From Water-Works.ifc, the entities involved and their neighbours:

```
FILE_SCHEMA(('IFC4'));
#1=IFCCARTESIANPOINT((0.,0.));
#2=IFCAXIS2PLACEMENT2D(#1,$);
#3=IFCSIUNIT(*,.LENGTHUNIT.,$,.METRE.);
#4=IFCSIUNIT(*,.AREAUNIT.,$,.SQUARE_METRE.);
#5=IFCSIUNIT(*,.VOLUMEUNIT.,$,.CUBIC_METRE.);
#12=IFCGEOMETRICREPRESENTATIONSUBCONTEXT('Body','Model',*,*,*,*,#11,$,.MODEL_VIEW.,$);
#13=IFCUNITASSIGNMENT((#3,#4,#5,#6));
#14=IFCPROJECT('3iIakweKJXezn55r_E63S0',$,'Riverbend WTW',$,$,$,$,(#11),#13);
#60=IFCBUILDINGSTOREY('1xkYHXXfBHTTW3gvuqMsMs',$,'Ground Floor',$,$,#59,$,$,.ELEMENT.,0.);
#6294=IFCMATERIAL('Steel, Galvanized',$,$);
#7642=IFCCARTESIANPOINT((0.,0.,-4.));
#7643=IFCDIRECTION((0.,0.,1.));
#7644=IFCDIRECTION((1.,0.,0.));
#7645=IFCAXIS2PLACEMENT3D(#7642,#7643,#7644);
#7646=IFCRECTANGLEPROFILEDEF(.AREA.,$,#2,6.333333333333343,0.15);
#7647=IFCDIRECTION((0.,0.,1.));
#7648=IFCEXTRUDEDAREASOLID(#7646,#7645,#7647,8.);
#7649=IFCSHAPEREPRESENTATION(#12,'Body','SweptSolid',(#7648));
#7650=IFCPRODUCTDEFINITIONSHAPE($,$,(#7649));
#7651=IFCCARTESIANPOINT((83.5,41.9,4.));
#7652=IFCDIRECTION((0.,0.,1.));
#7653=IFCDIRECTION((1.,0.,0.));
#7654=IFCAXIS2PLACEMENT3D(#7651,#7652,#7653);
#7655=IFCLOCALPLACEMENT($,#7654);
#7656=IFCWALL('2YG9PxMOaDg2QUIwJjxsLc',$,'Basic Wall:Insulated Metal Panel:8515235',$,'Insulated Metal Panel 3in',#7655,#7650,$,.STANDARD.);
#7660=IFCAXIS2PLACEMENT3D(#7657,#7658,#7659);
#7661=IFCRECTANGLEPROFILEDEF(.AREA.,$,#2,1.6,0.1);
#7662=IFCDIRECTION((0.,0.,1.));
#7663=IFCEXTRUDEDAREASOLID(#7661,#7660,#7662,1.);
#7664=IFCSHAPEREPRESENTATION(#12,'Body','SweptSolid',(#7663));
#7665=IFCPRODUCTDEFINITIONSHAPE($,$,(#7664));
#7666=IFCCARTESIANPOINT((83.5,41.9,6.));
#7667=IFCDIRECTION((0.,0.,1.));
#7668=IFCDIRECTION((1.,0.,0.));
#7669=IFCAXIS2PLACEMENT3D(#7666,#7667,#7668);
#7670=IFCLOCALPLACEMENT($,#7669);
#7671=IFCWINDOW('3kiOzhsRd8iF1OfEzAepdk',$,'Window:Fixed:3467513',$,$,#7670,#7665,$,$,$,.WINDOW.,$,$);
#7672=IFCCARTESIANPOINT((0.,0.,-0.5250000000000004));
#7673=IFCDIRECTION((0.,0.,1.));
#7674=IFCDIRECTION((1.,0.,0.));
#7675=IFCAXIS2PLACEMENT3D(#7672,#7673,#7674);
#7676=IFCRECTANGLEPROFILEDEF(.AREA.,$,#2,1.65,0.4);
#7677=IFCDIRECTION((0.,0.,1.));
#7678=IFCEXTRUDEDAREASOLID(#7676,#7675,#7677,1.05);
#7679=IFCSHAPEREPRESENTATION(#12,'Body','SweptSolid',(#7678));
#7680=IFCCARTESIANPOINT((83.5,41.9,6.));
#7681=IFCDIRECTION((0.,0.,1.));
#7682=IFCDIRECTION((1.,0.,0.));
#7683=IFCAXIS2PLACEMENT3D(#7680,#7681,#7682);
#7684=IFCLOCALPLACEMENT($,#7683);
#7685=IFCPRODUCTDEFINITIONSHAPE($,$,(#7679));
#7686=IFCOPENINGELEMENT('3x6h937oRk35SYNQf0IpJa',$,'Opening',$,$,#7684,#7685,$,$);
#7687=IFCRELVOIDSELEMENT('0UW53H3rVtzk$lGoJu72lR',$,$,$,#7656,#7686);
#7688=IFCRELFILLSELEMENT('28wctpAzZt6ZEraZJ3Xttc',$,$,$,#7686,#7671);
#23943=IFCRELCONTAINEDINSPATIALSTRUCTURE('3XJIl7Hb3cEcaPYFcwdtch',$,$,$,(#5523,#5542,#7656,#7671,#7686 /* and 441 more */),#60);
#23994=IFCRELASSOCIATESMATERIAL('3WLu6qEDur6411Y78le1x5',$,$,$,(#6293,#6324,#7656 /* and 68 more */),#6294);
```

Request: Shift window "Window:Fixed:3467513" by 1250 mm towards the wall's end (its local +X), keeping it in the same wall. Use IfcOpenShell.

```python
import ifcopenshell
import ifcopenshell.api.geometry
import ifcopenshell.util.placement
import ifcopenshell.util.unit

model = ifcopenshell.open("Water-Works.ifc")
unit_scale = ifcopenshell.util.unit.calculate_unit_scale(model)

window = model.by_guid("3kiOzhsRd8iF1OfEzAepdk")
opening = window.FillsVoids[0].RelatingOpeningElement
wall = opening.VoidsElements[0].RelatingBuildingElement

wall_matrix = ifcopenshell.util.placement.get_local_placement(wall.ObjectPlacement)
shift = wall_matrix[:3, 0] * 1.25 / unit_scale
before = ifcopenshell.util.placement.get_local_placement(window.ObjectPlacement)[:3, 3].copy()

# The window is not placed relative to its opening, so move both.
for product in (opening, window):
    matrix = ifcopenshell.util.placement.get_local_placement(product.ObjectPlacement)
    matrix[:3, 3] += shift
    ifcopenshell.api.geometry.edit_object_placement(model, product=product, matrix=matrix, is_si=False)

after = ifcopenshell.util.placement.get_local_placement(window.ObjectPlacement)[:3, 3]
print("window moved by", (after - before).round(3) + 0.0)

model.write("Water-Works-out.ifc")
```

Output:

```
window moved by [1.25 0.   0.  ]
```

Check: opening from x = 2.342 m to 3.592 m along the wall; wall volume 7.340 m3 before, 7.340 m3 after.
